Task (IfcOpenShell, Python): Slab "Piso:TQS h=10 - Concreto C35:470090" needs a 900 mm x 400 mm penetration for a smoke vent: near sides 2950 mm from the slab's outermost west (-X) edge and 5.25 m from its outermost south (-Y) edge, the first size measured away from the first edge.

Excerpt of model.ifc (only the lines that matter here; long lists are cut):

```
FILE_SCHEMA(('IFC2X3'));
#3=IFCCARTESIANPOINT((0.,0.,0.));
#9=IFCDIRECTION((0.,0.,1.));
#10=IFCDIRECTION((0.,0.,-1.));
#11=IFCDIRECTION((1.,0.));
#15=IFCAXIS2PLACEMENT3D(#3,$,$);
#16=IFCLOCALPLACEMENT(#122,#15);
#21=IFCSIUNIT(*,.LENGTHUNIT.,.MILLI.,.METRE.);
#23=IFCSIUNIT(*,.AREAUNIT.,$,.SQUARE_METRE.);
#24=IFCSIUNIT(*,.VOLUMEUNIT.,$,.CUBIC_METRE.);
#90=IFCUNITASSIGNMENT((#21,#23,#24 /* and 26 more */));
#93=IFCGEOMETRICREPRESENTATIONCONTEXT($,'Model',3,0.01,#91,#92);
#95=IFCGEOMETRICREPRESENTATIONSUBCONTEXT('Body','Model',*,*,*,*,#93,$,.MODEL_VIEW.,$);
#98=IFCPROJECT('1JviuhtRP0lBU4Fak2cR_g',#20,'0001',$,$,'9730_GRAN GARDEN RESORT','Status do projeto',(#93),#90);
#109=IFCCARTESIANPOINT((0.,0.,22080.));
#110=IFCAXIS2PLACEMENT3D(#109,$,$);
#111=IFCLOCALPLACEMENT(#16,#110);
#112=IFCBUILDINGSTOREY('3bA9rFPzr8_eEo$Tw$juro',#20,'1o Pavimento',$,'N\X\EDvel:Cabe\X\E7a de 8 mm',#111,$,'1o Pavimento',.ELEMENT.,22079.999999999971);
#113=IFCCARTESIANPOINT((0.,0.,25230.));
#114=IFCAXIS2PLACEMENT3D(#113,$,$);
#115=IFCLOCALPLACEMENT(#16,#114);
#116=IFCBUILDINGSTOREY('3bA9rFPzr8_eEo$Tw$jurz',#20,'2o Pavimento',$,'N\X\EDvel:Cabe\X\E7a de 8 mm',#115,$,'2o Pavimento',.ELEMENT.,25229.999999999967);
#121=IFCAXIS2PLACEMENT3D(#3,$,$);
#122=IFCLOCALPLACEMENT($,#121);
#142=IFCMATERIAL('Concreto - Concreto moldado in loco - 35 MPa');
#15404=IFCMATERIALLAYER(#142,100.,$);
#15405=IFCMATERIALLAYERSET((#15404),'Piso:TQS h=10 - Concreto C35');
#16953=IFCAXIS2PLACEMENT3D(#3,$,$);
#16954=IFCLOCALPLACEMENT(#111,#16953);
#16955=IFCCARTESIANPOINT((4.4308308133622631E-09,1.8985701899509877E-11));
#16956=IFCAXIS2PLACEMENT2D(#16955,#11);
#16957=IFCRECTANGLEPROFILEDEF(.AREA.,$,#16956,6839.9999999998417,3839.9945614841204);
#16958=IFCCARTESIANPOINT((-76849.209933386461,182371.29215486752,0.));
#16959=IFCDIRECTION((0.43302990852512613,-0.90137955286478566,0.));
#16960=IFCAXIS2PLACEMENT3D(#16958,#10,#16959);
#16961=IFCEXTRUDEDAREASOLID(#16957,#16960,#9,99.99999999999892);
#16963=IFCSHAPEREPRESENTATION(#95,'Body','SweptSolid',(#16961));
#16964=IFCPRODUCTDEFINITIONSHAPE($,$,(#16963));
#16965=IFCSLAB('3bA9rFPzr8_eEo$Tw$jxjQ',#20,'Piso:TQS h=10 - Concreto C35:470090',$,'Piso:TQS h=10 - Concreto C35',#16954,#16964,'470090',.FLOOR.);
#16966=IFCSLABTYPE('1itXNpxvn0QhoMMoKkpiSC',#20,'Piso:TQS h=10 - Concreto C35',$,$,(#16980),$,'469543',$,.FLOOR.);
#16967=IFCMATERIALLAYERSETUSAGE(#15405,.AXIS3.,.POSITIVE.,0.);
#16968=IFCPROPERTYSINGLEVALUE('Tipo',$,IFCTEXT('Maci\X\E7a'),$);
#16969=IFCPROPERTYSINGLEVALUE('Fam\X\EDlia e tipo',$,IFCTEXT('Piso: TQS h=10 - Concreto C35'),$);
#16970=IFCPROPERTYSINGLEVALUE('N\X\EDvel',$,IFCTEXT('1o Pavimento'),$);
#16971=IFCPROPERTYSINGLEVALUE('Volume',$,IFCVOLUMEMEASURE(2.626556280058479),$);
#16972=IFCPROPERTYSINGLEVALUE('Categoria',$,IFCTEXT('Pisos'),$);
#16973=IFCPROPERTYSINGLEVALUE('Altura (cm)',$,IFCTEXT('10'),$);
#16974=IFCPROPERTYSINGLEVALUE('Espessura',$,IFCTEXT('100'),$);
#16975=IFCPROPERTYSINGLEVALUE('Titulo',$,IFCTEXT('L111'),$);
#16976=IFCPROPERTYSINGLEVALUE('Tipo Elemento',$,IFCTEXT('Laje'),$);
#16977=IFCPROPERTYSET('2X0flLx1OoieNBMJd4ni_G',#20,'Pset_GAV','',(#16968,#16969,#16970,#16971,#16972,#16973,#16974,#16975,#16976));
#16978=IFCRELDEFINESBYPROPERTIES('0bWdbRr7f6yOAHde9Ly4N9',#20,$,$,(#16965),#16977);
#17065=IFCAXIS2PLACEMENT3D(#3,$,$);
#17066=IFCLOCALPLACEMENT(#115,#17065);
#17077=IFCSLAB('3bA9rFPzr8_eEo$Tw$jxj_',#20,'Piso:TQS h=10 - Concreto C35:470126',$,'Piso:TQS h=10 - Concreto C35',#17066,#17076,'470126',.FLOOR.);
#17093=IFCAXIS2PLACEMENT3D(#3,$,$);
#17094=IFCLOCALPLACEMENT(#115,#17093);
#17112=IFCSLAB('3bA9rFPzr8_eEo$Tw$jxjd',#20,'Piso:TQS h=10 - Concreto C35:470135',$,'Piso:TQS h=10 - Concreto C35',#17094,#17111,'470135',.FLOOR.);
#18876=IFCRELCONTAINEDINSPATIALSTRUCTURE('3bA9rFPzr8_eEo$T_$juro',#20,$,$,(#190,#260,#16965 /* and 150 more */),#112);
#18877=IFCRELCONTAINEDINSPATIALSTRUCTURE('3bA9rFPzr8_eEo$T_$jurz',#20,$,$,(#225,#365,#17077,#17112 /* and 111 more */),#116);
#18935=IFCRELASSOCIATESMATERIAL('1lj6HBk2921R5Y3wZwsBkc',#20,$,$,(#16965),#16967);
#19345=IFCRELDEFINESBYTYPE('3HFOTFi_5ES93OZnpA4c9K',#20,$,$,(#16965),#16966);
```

```python
import numpy as np
import ifcopenshell
import ifcopenshell.api.feature
import ifcopenshell.api.geometry
import ifcopenshell.api.pset
import ifcopenshell.api.root
import ifcopenshell.geom
import ifcopenshell.util.element
import ifcopenshell.util.placement
import ifcopenshell.util.representation
import ifcopenshell.util.shape
import ifcopenshell.util.unit

model = ifcopenshell.open("model.ifc")
unit_scale = ifcopenshell.util.unit.calculate_unit_scale(model)
volume_scale = ifcopenshell.util.unit.calculate_unit_scale(model, "VOLUMEUNIT")
settings = ifcopenshell.geom.settings()


def volume(element):
    """Net volume in cubic metres, openings subtracted."""
    shape = ifcopenshell.geom.create_shape(settings, element)
    return ifcopenshell.util.shape.get_volume(shape.geometry)


slab = model.by_id(16965)
before = volume(slab)

# Extent in the slab's own axes, in metres. The edges named are its -X and -Y sides.
slab_shape = ifcopenshell.geom.create_shape(settings, slab)
vertices = ifcopenshell.util.shape.get_vertices(slab_shape.geometry)
x_min, y_min, bottom = vertices.min(axis=0)
top = vertices[:, 2].max()

opening = ifcopenshell.api.root.create_entity(model, ifc_class="IfcOpeningElement", name="Smoke vent opening")
context = ifcopenshell.util.representation.get_context(model, "Model", "Body", "MODEL_VIEW")
width, depth = 0.9, 0.4
outline = [(0.0, 0.0), (width, 0.0), (width, depth), (0.0, depth), (0.0, 0.0)]
# Overshoot both faces by 50 mm so the cut is clean.
shape = ifcopenshell.api.geometry.add_slab_representation(
    model, context=context, depth=top - bottom + 0.1, polyline=outline
)
ifcopenshell.api.geometry.assign_representation(model, product=opening, representation=shape)

matrix = ifcopenshell.util.placement.get_local_placement(slab.ObjectPlacement)
matrix[:, 3] = matrix @ np.append(np.array([x_min + 2.95, y_min + 5.25, bottom - 0.05]) / unit_scale, 1.0)
ifcopenshell.api.geometry.edit_object_placement(model, product=opening, matrix=matrix, is_si=False)
ifcopenshell.api.feature.add_feature(model, feature=opening, element=slab)

after = volume(slab)

# Update the slab's stored quantities.
pset = model.by_id(ifcopenshell.util.element.get_pset(slab, "Pset_GAV", should_inherit=False)["id"])
ifcopenshell.api.pset.edit_pset(model, pset=pset, properties={
    "Volume": model.create_entity("IfcVolumeMeasure", after / volume_scale),
})

print(f"slab volume {before:.3f} -> {after:.3f} m3")

model.write("model_v2.ifc")
```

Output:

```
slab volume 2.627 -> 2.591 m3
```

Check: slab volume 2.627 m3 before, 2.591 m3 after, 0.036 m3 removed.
